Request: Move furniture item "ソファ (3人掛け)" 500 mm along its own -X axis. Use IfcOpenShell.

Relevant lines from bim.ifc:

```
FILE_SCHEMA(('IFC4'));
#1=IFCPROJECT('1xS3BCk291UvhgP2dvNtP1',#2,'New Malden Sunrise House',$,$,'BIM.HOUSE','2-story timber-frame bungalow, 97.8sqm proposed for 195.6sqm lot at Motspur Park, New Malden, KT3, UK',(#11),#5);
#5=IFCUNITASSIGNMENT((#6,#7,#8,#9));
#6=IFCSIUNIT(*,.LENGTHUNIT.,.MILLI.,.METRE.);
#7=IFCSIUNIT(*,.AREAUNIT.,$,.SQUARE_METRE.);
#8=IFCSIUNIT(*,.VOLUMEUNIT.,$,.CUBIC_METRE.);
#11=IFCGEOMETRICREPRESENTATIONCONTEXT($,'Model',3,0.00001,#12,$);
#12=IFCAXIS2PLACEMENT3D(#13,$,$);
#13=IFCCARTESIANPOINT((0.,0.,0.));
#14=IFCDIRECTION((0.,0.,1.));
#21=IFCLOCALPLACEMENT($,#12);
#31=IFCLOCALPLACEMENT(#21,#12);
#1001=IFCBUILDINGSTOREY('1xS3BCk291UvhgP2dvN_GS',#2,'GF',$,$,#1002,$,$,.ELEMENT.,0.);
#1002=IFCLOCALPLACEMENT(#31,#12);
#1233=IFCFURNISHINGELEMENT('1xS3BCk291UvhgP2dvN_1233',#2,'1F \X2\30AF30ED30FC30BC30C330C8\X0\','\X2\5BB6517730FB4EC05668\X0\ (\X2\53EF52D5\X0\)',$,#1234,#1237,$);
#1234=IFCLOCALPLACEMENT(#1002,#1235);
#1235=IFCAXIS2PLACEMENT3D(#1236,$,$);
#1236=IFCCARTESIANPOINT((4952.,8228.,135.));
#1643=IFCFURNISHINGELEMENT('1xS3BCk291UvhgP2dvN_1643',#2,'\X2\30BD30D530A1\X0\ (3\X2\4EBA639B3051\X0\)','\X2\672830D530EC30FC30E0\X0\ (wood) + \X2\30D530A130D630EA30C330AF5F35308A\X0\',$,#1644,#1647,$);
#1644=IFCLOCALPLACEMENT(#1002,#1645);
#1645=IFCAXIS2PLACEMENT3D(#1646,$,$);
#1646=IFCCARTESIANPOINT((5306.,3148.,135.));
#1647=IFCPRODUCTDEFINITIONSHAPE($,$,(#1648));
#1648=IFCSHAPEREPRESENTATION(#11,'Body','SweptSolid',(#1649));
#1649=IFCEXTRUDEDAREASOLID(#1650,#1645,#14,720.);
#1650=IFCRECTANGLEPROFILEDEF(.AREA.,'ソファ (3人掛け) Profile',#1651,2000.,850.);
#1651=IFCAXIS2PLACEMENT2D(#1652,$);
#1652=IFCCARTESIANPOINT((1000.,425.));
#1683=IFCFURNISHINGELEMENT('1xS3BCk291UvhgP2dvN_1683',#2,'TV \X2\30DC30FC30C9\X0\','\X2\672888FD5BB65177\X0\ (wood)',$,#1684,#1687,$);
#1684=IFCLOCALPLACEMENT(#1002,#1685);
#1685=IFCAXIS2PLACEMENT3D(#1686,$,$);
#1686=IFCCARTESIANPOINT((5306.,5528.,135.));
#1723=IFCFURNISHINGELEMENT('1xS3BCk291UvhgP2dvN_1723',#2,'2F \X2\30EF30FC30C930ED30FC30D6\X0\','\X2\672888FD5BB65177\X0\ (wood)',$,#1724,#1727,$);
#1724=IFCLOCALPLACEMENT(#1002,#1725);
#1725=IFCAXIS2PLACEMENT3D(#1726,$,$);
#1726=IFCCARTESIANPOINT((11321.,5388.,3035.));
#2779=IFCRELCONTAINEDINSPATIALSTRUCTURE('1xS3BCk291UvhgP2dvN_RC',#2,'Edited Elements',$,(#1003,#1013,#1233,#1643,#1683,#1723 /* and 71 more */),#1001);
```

```python
import ifcopenshell
import ifcopenshell.api.geometry
import ifcopenshell.util.placement

model = ifcopenshell.open("bim.ifc")

item = model.by_guid("1xS3BCk291UvhgP2dvN_1643")
matrix = ifcopenshell.util.placement.get_local_placement(item.ObjectPlacement)
matrix[:3, 3] -= matrix[:3, 0] * 500.0
ifcopenshell.api.geometry.edit_object_placement(model, product=item, matrix=matrix, is_si=False)

print(ifcopenshell.util.placement.get_local_placement(item.ObjectPlacement).round(3) + 0.0)

model.write("bim_edited.ifc")
```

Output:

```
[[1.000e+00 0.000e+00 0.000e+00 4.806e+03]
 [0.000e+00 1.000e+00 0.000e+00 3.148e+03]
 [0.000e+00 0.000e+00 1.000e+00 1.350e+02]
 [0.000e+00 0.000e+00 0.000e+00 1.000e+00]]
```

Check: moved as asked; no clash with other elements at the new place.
